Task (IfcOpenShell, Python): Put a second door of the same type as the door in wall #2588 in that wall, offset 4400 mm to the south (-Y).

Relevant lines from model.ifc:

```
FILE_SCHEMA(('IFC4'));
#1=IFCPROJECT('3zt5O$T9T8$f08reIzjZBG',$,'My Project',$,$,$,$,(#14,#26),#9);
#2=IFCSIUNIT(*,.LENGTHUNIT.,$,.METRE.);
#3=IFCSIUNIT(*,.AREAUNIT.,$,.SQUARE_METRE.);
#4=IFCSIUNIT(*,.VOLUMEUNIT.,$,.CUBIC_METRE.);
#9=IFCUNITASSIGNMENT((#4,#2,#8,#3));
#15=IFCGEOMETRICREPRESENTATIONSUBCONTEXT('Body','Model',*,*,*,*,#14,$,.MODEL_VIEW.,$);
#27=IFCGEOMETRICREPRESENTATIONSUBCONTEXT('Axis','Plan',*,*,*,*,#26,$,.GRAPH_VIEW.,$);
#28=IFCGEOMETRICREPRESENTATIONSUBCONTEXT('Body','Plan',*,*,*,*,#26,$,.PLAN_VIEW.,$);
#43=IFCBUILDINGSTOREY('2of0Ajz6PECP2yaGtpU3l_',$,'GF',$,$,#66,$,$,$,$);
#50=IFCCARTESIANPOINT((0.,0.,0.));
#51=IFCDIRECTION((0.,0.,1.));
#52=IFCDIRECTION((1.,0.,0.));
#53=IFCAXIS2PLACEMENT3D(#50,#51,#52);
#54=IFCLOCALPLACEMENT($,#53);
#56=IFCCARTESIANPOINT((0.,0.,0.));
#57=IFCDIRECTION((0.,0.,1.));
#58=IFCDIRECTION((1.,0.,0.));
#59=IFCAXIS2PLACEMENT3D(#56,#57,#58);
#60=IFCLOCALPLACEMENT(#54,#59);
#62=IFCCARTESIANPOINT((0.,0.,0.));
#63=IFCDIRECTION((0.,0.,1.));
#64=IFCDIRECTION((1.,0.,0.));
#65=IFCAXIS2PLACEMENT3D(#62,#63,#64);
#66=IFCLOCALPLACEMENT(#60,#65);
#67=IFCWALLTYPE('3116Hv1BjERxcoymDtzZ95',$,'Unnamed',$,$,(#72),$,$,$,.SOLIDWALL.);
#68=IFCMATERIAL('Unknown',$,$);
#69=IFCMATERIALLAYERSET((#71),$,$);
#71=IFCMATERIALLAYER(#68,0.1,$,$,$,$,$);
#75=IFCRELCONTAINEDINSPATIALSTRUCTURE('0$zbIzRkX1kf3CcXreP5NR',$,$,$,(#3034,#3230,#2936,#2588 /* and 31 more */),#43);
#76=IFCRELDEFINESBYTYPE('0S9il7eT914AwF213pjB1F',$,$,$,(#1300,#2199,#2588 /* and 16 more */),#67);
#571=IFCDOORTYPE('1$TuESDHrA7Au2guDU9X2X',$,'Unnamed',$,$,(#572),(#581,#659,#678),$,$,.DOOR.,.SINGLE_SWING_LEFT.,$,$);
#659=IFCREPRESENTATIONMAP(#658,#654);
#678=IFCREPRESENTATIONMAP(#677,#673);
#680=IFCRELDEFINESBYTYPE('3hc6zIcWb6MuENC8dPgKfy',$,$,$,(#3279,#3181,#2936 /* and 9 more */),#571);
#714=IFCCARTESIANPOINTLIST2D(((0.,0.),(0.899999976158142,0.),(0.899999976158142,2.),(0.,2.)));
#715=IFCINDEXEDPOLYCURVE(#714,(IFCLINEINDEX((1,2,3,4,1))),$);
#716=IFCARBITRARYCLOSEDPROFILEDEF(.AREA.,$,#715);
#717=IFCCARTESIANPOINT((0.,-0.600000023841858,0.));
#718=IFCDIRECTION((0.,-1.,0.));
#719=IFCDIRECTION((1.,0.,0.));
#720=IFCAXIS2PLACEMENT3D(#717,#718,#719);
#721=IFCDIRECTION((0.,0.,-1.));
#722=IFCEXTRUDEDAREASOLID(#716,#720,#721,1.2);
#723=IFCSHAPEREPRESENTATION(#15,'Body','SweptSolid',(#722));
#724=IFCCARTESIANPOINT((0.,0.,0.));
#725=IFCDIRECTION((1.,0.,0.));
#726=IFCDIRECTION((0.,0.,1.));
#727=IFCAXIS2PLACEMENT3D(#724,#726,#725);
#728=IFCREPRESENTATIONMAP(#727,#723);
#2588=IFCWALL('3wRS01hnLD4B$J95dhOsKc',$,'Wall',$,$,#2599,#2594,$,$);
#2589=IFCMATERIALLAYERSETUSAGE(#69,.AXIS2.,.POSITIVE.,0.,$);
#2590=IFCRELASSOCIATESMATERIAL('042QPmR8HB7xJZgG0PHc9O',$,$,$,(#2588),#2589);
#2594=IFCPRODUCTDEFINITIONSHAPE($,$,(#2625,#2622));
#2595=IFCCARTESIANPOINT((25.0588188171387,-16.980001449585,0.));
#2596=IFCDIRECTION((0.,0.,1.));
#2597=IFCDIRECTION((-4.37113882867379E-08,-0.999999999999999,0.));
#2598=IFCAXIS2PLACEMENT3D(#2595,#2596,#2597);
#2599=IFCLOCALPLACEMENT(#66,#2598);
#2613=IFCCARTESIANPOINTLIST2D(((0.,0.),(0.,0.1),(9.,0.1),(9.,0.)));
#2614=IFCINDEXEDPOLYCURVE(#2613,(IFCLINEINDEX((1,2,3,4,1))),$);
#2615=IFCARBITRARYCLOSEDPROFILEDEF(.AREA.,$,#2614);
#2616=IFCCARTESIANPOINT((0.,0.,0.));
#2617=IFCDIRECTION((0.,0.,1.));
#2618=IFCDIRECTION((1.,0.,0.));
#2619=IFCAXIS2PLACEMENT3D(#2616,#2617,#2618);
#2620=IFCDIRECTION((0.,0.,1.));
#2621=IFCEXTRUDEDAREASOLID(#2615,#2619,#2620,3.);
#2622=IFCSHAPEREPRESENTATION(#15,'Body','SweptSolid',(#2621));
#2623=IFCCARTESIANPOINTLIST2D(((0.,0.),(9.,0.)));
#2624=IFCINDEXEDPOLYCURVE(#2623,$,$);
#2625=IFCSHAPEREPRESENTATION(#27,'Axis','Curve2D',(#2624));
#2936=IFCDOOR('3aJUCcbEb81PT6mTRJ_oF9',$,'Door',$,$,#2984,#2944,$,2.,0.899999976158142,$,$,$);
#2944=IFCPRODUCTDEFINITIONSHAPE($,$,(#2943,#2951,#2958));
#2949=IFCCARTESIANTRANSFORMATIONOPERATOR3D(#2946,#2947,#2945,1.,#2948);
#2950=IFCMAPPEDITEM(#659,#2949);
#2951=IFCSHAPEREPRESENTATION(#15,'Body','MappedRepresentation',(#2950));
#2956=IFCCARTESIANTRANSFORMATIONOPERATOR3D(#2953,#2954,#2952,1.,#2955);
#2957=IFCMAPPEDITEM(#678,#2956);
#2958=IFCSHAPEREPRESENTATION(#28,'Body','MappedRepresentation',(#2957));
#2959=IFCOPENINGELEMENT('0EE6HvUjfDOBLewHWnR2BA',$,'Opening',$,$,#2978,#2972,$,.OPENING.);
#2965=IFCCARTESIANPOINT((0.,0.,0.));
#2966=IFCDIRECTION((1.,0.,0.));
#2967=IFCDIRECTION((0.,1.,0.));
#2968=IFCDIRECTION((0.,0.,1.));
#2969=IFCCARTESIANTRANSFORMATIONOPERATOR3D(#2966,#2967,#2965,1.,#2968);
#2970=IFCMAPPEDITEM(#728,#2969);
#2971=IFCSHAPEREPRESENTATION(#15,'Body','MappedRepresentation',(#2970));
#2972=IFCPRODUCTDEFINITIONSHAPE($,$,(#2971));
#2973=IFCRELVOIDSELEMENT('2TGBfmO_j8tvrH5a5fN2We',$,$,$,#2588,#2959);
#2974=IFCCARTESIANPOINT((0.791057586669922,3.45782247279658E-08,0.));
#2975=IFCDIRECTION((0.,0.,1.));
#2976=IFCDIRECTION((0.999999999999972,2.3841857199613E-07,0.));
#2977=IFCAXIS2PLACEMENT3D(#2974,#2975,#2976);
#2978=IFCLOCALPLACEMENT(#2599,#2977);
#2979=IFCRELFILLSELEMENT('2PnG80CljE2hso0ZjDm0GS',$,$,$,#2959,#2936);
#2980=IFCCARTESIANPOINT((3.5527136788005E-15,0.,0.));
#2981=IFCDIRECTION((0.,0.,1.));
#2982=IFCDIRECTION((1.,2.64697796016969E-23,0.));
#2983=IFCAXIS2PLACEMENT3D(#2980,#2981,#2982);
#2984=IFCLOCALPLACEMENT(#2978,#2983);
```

```python
import ifcopenshell
import ifcopenshell.api.feature
import ifcopenshell.api.geometry
import ifcopenshell.api.root
import ifcopenshell.geom
import ifcopenshell.util.element
import ifcopenshell.util.placement
import ifcopenshell.util.shape
import ifcopenshell.util.unit

model = ifcopenshell.open("model.ifc")
unit_scale = ifcopenshell.util.unit.calculate_unit_scale(model)
settings = ifcopenshell.geom.settings()


def volume(element):
    """Net volume in cubic metres, openings subtracted."""
    shape = ifcopenshell.geom.create_shape(settings, element)
    return ifcopenshell.util.shape.get_volume(shape.geometry)


door = model.by_id(2936)
opening = door.FillsVoids[0].RelatingOpeningElement
wall = opening.VoidsElements[0].RelatingBuildingElement
before = volume(wall)
shift = ifcopenshell.util.placement.get_local_placement(wall.ObjectPlacement)[:3, 0] * 4.4 / unit_scale

# copy_class copies the void relationship, type, container and properties, but no geometry.
new_opening = ifcopenshell.api.root.copy_class(model, product=opening)
new_opening.Representation = ifcopenshell.util.element.copy_deep(
    model, opening.Representation, exclude=["IfcGeometricRepresentationContext", "IfcRepresentationMap"]
)
new_door = ifcopenshell.api.root.copy_class(model, product=door)
new_door.Representation = ifcopenshell.util.element.copy_deep(
    model, door.Representation, exclude=["IfcGeometricRepresentationContext", "IfcRepresentationMap"]
)
ifcopenshell.api.feature.add_filling(model, opening=new_opening, element=new_door)

for old, new in ((opening, new_opening), (door, new_door)):
    matrix = ifcopenshell.util.placement.get_local_placement(old.ObjectPlacement)
    matrix[:3, 3] += shift
    ifcopenshell.api.geometry.edit_object_placement(model, product=new, matrix=matrix, is_si=False)

after = volume(wall)

print(f"wall volume {before:.3f} -> {after:.3f} m3")

model.write("model_v2.ifc")
```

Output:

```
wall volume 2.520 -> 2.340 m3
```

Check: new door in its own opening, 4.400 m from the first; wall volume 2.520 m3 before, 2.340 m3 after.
